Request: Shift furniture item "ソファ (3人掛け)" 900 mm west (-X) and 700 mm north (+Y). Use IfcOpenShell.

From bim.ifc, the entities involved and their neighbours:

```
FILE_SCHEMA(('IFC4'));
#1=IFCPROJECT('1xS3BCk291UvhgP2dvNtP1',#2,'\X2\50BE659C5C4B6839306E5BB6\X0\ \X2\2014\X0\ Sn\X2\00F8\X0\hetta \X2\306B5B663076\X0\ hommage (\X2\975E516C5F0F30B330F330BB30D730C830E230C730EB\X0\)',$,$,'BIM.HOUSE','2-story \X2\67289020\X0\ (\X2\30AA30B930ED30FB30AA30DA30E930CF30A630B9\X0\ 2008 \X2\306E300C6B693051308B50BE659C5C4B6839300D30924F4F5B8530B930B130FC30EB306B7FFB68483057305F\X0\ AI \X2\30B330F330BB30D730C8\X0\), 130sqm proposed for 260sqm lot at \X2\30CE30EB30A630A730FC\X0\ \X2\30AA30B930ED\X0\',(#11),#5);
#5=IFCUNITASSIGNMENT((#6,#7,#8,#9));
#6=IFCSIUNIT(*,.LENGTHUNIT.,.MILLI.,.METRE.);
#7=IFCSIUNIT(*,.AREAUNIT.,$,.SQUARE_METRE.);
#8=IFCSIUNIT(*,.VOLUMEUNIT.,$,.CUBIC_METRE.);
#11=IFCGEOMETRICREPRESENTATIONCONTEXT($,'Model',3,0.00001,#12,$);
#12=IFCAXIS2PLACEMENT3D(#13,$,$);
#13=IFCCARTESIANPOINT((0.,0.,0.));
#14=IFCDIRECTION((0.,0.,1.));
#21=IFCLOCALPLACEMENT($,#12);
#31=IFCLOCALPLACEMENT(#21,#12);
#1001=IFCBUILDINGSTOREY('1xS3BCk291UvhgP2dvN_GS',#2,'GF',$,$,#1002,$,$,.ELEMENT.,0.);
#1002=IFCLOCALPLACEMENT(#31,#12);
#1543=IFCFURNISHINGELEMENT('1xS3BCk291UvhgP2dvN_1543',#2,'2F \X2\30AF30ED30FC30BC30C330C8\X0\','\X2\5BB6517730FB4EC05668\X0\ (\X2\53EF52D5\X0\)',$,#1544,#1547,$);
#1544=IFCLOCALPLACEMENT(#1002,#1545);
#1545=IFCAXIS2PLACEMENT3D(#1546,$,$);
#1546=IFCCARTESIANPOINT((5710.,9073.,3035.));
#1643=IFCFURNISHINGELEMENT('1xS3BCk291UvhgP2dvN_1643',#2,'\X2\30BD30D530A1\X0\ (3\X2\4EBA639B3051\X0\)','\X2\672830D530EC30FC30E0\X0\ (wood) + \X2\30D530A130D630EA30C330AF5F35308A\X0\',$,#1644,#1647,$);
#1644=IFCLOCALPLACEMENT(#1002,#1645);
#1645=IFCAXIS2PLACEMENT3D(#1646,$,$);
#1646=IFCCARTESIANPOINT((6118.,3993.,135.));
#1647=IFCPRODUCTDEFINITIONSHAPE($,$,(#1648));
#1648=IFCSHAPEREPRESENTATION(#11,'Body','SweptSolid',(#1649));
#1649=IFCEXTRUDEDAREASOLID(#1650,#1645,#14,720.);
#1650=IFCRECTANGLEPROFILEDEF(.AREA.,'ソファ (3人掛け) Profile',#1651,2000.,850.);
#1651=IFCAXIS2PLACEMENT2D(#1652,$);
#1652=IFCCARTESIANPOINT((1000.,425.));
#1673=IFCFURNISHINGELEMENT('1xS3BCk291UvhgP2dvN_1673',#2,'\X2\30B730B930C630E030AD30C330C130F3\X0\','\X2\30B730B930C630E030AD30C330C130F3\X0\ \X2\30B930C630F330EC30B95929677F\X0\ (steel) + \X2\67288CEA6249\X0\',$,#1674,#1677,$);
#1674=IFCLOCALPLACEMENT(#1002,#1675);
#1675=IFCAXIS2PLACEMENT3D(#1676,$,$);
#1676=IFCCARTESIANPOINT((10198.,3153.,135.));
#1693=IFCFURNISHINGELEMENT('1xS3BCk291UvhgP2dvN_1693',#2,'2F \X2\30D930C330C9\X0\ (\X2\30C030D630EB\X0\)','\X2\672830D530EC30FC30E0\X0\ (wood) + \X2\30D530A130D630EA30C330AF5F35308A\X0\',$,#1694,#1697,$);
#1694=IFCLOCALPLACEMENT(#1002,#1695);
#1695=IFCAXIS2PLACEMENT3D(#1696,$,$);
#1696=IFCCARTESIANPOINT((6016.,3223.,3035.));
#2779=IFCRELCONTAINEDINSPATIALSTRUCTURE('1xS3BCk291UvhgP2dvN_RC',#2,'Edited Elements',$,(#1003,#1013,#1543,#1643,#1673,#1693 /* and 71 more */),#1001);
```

```python
import ifcopenshell
import ifcopenshell.api.geometry
import ifcopenshell.util.placement

model = ifcopenshell.open("bim.ifc")

item = model.by_id(1643)
matrix = ifcopenshell.util.placement.get_local_placement(item.ObjectPlacement)
matrix[0, 3] -= 900.0
matrix[1, 3] += 700.0
ifcopenshell.api.geometry.edit_object_placement(model, product=item, matrix=matrix, is_si=False)

print(ifcopenshell.util.placement.get_local_placement(item.ObjectPlacement).round(3) + 0.0)

model.write("bim-out.ifc")
```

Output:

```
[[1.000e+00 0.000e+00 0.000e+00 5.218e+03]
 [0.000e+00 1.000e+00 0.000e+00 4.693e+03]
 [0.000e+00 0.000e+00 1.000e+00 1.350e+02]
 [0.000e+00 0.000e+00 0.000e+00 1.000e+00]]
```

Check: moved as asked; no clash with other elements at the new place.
